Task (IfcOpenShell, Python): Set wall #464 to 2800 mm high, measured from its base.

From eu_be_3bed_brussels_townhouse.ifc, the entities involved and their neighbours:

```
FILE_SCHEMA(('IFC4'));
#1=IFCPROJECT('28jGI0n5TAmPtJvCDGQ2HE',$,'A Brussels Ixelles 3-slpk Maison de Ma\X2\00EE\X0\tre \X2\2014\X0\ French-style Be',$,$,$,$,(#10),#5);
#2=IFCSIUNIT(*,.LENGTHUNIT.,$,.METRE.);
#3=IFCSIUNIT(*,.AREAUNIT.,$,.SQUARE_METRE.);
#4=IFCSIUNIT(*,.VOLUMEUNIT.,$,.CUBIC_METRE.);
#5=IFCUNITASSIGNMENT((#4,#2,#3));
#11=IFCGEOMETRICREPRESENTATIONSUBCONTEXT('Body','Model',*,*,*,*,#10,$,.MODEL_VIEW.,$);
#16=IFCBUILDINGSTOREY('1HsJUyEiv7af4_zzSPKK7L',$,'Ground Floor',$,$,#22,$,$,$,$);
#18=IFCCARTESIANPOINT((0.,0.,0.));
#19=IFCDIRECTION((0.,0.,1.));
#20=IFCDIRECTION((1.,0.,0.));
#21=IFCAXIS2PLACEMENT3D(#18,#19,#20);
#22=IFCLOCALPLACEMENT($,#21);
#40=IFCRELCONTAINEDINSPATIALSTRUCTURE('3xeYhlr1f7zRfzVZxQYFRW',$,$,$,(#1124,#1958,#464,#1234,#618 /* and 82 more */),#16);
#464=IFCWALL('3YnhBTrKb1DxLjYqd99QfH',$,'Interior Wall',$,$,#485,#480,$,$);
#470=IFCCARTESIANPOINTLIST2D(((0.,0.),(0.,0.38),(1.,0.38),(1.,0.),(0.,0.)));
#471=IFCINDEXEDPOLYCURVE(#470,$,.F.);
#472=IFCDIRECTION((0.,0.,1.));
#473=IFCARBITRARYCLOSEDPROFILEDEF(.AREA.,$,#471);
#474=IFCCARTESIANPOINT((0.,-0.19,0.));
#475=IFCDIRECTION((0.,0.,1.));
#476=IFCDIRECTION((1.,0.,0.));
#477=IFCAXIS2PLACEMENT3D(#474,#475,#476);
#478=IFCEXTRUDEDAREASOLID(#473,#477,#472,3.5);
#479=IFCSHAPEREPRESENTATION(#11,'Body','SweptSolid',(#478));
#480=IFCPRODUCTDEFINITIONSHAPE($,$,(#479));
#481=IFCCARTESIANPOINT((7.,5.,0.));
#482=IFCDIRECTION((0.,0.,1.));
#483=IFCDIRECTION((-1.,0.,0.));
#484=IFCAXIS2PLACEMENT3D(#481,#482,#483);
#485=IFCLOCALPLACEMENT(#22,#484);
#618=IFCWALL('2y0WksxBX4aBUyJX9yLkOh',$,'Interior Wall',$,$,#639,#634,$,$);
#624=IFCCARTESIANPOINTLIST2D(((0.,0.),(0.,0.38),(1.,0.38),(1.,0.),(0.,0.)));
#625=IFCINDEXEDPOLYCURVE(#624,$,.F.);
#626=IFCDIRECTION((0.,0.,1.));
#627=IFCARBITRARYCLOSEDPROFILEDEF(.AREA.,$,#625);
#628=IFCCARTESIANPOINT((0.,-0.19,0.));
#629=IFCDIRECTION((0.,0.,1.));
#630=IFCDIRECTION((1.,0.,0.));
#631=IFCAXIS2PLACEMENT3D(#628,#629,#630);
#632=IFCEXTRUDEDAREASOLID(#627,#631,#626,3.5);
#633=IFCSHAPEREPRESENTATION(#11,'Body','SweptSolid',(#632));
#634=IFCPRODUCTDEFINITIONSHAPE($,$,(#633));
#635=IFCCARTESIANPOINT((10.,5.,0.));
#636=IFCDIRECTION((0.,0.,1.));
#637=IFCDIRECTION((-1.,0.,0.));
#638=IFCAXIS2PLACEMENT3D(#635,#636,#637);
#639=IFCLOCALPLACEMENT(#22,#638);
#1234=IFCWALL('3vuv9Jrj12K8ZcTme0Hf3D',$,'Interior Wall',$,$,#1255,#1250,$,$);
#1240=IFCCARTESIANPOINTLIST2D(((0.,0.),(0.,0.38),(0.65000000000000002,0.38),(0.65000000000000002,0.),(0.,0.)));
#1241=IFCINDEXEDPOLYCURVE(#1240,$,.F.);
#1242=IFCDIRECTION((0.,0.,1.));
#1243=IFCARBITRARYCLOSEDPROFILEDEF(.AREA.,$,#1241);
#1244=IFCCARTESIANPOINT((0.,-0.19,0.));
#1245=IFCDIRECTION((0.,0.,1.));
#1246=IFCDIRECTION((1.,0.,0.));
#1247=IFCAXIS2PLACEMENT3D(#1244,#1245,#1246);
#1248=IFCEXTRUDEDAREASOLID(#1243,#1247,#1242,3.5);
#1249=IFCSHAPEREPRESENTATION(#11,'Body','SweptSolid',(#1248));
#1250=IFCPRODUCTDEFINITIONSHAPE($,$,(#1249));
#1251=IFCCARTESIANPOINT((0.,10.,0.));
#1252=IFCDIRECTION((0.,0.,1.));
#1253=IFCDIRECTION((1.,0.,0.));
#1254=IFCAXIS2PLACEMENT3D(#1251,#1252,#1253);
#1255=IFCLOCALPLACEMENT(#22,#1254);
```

```python
import ifcopenshell
import ifcopenshell.geom
import ifcopenshell.util.representation
import ifcopenshell.util.shape
import ifcopenshell.util.unit

model = ifcopenshell.open("eu_be_3bed_brussels_townhouse.ifc")
unit_scale = ifcopenshell.util.unit.calculate_unit_scale(model)
settings = ifcopenshell.geom.settings()


def volume(element):
    """Net volume in cubic metres, openings subtracted."""
    shape = ifcopenshell.geom.create_shape(settings, element)
    return ifcopenshell.util.shape.get_volume(shape.geometry)


wall = model.by_id(464)
before = volume(wall)

body = ifcopenshell.util.representation.get_representation(wall, "Model", "Body")
solid = body.Items[0]
old_height = solid.Depth
solid.Depth = 2.8 / unit_scale
after = volume(wall)

print(f"height {old_height:g} -> {solid.Depth:g}, volume {before:.3f} -> {after:.3f} m3")

model.write("eu_be_3bed_brussels_townhouse_edited.ifc")
```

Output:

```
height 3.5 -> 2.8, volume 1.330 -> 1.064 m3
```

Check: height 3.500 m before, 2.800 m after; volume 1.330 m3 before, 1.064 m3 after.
